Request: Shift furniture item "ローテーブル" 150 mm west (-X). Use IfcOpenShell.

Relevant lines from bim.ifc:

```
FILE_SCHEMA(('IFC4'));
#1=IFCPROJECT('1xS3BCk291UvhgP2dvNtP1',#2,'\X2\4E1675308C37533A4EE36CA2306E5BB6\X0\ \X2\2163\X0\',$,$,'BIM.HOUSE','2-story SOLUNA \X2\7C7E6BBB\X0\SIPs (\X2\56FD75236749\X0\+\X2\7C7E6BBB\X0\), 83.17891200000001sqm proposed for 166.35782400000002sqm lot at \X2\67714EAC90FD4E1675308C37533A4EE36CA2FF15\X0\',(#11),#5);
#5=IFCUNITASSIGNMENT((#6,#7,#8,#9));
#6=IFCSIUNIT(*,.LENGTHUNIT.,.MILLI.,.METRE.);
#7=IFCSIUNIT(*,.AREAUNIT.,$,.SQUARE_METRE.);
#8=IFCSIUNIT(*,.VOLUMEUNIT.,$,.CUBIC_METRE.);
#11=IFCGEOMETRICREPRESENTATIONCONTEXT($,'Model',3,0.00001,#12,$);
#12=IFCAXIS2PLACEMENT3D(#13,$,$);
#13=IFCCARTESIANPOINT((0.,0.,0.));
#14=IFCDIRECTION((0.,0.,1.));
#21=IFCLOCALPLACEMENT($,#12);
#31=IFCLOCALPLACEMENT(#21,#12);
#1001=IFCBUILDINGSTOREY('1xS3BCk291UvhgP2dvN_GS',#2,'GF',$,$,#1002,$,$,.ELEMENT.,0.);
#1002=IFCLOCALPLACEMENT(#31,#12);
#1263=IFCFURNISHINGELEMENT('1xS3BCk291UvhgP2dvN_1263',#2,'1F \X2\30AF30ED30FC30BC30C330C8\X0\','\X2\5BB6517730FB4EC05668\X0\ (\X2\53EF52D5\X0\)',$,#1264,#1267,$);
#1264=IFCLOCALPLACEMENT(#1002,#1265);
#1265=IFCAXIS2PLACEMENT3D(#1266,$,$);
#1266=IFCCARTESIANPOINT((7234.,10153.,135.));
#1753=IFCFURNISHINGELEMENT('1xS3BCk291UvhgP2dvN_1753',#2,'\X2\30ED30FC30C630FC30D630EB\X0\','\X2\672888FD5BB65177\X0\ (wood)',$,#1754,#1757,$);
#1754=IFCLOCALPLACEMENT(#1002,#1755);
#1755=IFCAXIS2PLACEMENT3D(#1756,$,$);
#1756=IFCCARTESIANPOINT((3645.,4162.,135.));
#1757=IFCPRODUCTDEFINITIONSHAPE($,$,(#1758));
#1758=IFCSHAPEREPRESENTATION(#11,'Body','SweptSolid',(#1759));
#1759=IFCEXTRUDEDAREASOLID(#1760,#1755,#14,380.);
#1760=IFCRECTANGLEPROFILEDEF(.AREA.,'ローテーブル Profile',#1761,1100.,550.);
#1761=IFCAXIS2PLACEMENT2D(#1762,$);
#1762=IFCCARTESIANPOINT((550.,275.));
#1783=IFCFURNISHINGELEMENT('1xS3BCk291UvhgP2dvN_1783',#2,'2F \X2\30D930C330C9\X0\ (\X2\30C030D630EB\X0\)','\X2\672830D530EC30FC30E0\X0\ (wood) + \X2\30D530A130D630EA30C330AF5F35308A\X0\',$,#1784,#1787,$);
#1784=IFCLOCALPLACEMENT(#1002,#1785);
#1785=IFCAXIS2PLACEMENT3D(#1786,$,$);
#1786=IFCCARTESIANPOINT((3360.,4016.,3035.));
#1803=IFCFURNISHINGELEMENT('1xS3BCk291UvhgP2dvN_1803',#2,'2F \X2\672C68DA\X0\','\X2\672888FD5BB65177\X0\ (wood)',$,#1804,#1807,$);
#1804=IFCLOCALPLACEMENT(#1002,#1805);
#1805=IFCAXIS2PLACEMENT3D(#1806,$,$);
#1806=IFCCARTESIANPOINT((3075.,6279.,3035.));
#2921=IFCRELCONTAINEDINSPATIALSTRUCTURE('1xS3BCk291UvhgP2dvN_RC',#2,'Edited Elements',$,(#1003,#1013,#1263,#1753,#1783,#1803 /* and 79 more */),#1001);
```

```python
import ifcopenshell
import ifcopenshell.api.geometry
import ifcopenshell.util.placement
import ifcopenshell.util.unit

model = ifcopenshell.open("bim.ifc")
unit_scale = ifcopenshell.util.unit.calculate_unit_scale(model)

item = model.by_guid("1xS3BCk291UvhgP2dvN_1753")
matrix = ifcopenshell.util.placement.get_local_placement(item.ObjectPlacement)
matrix[0, 3] -= 0.15 / unit_scale
ifcopenshell.api.geometry.edit_object_placement(model, product=item, matrix=matrix, is_si=False)

print(ifcopenshell.util.placement.get_local_placement(item.ObjectPlacement).round(3) + 0.0)

model.write("bim-out.ifc")
```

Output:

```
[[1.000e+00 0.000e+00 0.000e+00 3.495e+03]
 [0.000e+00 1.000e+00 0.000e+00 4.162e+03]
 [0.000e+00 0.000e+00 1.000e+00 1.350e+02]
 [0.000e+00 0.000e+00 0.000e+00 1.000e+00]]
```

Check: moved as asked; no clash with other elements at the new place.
